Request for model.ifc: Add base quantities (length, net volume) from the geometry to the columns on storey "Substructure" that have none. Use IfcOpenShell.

First a look at what the model holds.

```python
import ifcopenshell
import ifcopenshell.util.element
import ifcopenshell.util.unit

model = ifcopenshell.open("model.ifc")
print(model.schema)
for unit_type in ("LENGTHUNIT", "AREAUNIT", "VOLUMEUNIT"):
    print(unit_type, ifcopenshell.util.unit.calculate_unit_scale(model, unit_type))
storey = next(s for s in model.by_type("IfcBuildingStorey") if s.Name == "Substructure")
columns = [e for e in ifcopenshell.util.element.get_decomposition(storey) if e.is_a("IfcColumn")]
for e in sorted(columns, key=lambda e: e.id()):
    print(e.id(), e.is_a(), e.Name, list(ifcopenshell.util.element.get_psets(e, qtos_only=True)), sep=" | ")
```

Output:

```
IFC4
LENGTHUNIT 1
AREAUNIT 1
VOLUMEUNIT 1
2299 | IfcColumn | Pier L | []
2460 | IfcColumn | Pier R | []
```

```python
import ifcopenshell
import ifcopenshell.api.pset
import ifcopenshell.geom
import ifcopenshell.util.element
import ifcopenshell.util.shape
import ifcopenshell.util.unit

model = ifcopenshell.open("model.ifc")
unit_scale = ifcopenshell.util.unit.calculate_unit_scale(model)
volume_scale = ifcopenshell.util.unit.calculate_unit_scale(model, "VOLUMEUNIT")
settings = ifcopenshell.geom.settings()

storey = next(s for s in model.by_type("IfcBuildingStorey") if s.Name == "Substructure")
columns = [e for e in ifcopenshell.util.element.get_decomposition(storey) if e.is_a("IfcColumn")]

for e in sorted(columns, key=lambda e: e.id()):
    if ifcopenshell.util.element.get_psets(e, qtos_only=True, should_inherit=False):
        continue
    # Geometry comes back in metres, in the element's own axes.
    shape = ifcopenshell.geom.create_shape(settings, e)
    values = {
        "Length": ifcopenshell.util.shape.get_z(shape.geometry) / unit_scale,
        "NetVolume": ifcopenshell.util.shape.get_volume(shape.geometry) / volume_scale,
    }
    qto = ifcopenshell.api.pset.add_qto(model, product=e, name="Qto_ColumnBaseQuantities")
    ifcopenshell.api.pset.edit_qto(model, qto=qto, properties=values)
    print(e.id(), {k: round(v, 3) for k, v in values.items()})

model.write("model_v2.ifc")
```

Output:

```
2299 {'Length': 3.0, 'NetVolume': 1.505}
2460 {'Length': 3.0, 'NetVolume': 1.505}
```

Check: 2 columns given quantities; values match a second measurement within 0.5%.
